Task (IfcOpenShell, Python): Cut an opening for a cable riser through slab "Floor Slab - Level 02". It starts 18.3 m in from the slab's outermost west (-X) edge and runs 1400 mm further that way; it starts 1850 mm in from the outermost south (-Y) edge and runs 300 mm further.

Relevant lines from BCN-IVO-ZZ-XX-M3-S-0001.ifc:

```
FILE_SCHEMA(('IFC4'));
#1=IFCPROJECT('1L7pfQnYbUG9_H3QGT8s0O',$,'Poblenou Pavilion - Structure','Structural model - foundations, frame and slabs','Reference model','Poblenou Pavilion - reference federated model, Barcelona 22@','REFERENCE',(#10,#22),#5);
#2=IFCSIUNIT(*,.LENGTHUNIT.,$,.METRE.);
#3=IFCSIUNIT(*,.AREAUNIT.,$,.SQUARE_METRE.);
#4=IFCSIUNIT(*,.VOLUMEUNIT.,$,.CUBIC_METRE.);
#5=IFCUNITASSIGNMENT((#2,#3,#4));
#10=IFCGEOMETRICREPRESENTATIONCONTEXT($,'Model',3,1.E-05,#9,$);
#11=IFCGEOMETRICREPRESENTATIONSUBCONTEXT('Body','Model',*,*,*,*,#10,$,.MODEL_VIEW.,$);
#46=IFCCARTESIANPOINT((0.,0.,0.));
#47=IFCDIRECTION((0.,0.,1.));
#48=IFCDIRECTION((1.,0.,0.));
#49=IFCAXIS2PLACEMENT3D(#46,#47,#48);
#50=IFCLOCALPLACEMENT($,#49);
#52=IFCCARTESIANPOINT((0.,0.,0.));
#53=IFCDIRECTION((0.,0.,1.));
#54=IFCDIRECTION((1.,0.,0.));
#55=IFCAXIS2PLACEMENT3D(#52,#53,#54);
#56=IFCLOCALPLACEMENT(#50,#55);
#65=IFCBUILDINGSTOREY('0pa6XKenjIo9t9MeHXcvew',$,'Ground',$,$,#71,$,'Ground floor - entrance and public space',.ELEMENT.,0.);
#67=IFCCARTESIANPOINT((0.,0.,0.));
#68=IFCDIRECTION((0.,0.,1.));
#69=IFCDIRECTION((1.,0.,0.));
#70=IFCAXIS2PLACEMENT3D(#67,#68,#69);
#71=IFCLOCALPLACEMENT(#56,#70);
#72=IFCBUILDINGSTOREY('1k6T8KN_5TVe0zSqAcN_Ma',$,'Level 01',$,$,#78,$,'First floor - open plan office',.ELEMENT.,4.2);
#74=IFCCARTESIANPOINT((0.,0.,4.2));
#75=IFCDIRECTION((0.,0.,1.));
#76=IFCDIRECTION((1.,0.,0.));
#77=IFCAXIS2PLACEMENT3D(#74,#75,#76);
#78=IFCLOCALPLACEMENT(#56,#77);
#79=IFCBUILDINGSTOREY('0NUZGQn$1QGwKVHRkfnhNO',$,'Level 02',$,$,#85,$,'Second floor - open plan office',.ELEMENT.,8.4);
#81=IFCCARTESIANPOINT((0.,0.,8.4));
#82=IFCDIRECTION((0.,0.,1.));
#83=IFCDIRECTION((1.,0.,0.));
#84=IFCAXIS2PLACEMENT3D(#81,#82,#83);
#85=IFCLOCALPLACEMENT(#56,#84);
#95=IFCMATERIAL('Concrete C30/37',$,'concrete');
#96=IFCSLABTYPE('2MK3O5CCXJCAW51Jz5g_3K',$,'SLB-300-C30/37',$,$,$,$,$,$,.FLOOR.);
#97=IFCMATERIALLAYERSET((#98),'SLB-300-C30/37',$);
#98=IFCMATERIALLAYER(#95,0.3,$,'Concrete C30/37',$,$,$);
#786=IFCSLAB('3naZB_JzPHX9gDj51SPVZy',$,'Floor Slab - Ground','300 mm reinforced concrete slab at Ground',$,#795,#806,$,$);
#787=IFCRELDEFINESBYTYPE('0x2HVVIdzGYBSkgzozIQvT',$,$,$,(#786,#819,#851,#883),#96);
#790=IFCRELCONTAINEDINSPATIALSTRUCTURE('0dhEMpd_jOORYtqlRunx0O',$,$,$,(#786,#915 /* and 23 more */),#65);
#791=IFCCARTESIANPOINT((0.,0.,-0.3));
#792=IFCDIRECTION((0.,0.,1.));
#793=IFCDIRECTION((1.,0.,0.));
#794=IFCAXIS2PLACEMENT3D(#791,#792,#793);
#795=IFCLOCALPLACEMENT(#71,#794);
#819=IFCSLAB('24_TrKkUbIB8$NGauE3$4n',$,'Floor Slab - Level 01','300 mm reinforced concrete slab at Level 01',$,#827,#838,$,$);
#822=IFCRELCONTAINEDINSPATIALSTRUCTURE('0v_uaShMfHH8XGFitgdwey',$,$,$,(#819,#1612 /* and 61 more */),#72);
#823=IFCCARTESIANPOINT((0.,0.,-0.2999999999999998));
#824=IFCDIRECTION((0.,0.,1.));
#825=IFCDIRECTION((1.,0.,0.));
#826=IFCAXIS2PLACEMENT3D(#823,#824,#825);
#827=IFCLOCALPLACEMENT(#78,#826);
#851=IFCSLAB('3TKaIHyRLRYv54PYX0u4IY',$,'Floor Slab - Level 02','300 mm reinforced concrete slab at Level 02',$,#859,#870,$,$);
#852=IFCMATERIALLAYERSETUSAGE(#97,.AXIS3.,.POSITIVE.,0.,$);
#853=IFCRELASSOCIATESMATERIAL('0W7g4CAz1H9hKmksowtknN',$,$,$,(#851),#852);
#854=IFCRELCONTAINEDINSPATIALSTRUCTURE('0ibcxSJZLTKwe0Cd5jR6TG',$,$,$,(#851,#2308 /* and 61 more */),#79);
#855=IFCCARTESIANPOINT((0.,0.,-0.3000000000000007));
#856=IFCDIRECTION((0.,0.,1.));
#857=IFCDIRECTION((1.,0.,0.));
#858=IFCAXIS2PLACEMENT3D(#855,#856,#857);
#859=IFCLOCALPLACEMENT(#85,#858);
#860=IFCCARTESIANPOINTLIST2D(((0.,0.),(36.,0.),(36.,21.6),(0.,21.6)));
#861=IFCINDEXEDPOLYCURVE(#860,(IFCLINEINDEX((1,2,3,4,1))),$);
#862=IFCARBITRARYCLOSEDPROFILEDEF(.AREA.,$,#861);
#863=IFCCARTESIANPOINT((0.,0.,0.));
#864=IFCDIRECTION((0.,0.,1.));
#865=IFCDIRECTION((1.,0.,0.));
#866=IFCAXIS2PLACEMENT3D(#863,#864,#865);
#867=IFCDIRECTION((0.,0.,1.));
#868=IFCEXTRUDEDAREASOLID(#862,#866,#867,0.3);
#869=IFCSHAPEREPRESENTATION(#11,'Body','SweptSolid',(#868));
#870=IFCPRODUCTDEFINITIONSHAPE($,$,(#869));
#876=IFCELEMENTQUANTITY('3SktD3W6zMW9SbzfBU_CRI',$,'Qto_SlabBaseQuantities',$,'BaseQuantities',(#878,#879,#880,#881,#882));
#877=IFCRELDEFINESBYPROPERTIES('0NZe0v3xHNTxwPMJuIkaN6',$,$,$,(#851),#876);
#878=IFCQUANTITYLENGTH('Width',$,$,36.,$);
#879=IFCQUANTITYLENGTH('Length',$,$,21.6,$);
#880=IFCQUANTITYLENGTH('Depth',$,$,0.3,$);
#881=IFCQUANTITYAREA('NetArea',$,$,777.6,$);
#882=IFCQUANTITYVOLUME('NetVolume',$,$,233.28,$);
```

```python
import numpy as np
import ifcopenshell
import ifcopenshell.api.feature
import ifcopenshell.api.geometry
import ifcopenshell.api.pset
import ifcopenshell.api.root
import ifcopenshell.geom
import ifcopenshell.util.element
import ifcopenshell.util.placement
import ifcopenshell.util.representation
import ifcopenshell.util.shape
import ifcopenshell.util.unit

model = ifcopenshell.open("BCN-IVO-ZZ-XX-M3-S-0001.ifc")
unit_scale = ifcopenshell.util.unit.calculate_unit_scale(model)
area_scale = ifcopenshell.util.unit.calculate_unit_scale(model, "AREAUNIT")
volume_scale = ifcopenshell.util.unit.calculate_unit_scale(model, "VOLUMEUNIT")
settings = ifcopenshell.geom.settings()


def volume(element):
    """Net volume in cubic metres, openings subtracted."""
    shape = ifcopenshell.geom.create_shape(settings, element)
    return ifcopenshell.util.shape.get_volume(shape.geometry)


slab = model.by_id(851)
before = volume(slab)

# Extent in the slab's own axes, in metres. The edges named are its -X and -Y sides.
slab_shape = ifcopenshell.geom.create_shape(settings, slab)
vertices = ifcopenshell.util.shape.get_vertices(slab_shape.geometry)
x_min, y_min, bottom = vertices.min(axis=0)
top = vertices[:, 2].max()

opening = ifcopenshell.api.root.create_entity(model, ifc_class="IfcOpeningElement", name="Cable riser opening", predefined_type="OPENING")
context = ifcopenshell.util.representation.get_context(model, "Model", "Body", "MODEL_VIEW")
width, depth = 1.4, 0.3
outline = [(0.0, 0.0), (width, 0.0), (width, depth), (0.0, depth), (0.0, 0.0)]
# Overshoot both faces by 50 mm so the cut is clean.
shape = ifcopenshell.api.geometry.add_slab_representation(
    model, context=context, depth=top - bottom + 0.1, polyline=outline
)
ifcopenshell.api.geometry.assign_representation(model, product=opening, representation=shape)

matrix = ifcopenshell.util.placement.get_local_placement(slab.ObjectPlacement)
matrix[:, 3] = matrix @ np.append(np.array([x_min + 18.3, y_min + 1.85, bottom - 0.05]) / unit_scale, 1.0)
ifcopenshell.api.geometry.edit_object_placement(model, product=opening, matrix=matrix, is_si=False)
ifcopenshell.api.feature.add_feature(model, feature=opening, element=slab)

after = volume(slab)

# Update the slab's stored quantities.
qto = model.by_id(ifcopenshell.util.element.get_pset(slab, "Qto_SlabBaseQuantities", should_inherit=False)["id"])
ifcopenshell.api.pset.edit_qto(model, qto=qto, properties={
    "NetArea": after / (top - bottom) / area_scale,
    "NetVolume": after / volume_scale,
})

print(f"slab volume {before:.3f} -> {after:.3f} m3")

model.write("BCN-IVO-ZZ-XX-M3-S-0001_rev.ifc")
```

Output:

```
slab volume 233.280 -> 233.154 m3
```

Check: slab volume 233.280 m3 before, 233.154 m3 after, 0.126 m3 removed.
